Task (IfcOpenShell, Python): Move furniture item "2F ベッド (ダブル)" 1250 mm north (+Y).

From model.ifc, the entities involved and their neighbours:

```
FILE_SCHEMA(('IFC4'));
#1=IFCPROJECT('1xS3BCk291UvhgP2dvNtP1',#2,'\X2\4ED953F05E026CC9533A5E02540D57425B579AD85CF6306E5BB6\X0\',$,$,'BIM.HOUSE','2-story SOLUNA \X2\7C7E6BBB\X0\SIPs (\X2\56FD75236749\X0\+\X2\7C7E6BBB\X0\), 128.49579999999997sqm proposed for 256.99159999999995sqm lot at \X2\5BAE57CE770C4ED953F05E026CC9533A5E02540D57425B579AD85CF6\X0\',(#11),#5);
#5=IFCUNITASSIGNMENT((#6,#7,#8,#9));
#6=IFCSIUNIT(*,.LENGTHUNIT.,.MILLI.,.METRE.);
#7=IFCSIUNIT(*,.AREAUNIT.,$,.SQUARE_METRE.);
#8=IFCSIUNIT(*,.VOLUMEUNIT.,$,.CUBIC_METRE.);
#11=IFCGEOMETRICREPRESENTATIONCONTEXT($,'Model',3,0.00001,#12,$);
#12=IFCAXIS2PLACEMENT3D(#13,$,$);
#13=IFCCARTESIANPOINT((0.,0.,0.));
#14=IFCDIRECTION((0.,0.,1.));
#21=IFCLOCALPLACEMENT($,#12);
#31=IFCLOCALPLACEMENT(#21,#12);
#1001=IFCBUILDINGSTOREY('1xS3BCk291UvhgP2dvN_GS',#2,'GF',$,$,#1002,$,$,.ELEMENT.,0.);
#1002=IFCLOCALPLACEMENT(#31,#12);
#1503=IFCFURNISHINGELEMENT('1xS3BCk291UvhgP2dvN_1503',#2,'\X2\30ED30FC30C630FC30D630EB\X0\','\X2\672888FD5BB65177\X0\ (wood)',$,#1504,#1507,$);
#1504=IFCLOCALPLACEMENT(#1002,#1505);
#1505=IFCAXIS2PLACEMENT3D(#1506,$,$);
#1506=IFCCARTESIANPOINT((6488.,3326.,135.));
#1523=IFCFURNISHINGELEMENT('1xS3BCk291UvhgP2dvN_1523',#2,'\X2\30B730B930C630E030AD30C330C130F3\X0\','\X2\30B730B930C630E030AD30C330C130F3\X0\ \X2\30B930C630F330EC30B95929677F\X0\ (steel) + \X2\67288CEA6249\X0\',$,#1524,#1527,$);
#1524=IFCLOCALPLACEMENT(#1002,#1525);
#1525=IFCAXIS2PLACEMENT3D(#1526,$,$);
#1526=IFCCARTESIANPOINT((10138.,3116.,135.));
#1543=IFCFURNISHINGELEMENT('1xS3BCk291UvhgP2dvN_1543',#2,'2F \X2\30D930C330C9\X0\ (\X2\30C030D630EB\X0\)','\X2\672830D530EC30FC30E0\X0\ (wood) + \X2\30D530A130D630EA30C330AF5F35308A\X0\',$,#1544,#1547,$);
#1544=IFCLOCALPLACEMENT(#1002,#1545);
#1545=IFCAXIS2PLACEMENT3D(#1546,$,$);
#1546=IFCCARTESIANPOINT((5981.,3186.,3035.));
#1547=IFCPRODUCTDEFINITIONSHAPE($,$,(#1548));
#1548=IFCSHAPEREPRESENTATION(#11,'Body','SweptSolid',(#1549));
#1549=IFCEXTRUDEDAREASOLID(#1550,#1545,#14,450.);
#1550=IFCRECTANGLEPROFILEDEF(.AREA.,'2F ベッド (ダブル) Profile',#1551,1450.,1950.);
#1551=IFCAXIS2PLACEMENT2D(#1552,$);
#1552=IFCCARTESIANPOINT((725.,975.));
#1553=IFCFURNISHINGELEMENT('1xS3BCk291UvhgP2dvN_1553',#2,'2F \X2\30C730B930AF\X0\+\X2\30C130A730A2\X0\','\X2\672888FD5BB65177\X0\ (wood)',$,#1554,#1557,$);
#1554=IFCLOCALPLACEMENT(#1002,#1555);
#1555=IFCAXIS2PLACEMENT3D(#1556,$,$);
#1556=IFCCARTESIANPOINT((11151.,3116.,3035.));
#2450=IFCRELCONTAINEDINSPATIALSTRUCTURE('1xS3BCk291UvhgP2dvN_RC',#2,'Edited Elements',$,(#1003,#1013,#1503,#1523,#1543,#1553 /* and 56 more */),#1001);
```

```python
import ifcopenshell
import ifcopenshell.api.geometry
import ifcopenshell.util.placement
import ifcopenshell.util.unit

model = ifcopenshell.open("model.ifc")
unit_scale = ifcopenshell.util.unit.calculate_unit_scale(model)

item = model.by_guid("1xS3BCk291UvhgP2dvN_1543")
matrix = ifcopenshell.util.placement.get_local_placement(item.ObjectPlacement)
matrix[1, 3] += 1.25 / unit_scale
ifcopenshell.api.geometry.edit_object_placement(model, product=item, matrix=matrix, is_si=False)

print(ifcopenshell.util.placement.get_local_placement(item.ObjectPlacement).round(3) + 0.0)

model.write("model-out.ifc")
```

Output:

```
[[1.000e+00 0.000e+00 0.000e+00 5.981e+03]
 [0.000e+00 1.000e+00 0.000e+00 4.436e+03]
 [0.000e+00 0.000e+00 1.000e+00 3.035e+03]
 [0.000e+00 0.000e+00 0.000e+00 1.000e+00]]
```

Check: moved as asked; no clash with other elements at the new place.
